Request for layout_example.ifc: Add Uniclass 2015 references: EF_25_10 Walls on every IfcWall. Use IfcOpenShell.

First a look at what the model holds.

```python
import ifcopenshell

model = ifcopenshell.open("layout_example.ifc")
print(model.schema)
print("classifications:", [c.Name for c in model.by_type("IfcClassification")])
for ifc_class in ("IfcDoor", "IfcRoof", "IfcStair", "IfcWall", "IfcWindow"):
    print(ifc_class, len(model.by_type(ifc_class)))
```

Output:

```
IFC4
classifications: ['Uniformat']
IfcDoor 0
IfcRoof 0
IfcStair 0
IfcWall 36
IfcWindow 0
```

```python
import ifcopenshell
import ifcopenshell.api.classification

model = ifcopenshell.open("layout_example.ifc")

system = ifcopenshell.api.classification.add_classification(model, classification="Uniclass 2015")

codes = {
    "IfcWall": ("EF_25_10", "Walls"),
}
for ifc_class, (code, name) in codes.items():
    products = model.by_type(ifc_class)
    ifcopenshell.api.classification.add_reference(
        model, products=products, classification=system, identification=code, name=name
    )
    print(code, len(products))

model.write("layout_example_updated.ifc")
```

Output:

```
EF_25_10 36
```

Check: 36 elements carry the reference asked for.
